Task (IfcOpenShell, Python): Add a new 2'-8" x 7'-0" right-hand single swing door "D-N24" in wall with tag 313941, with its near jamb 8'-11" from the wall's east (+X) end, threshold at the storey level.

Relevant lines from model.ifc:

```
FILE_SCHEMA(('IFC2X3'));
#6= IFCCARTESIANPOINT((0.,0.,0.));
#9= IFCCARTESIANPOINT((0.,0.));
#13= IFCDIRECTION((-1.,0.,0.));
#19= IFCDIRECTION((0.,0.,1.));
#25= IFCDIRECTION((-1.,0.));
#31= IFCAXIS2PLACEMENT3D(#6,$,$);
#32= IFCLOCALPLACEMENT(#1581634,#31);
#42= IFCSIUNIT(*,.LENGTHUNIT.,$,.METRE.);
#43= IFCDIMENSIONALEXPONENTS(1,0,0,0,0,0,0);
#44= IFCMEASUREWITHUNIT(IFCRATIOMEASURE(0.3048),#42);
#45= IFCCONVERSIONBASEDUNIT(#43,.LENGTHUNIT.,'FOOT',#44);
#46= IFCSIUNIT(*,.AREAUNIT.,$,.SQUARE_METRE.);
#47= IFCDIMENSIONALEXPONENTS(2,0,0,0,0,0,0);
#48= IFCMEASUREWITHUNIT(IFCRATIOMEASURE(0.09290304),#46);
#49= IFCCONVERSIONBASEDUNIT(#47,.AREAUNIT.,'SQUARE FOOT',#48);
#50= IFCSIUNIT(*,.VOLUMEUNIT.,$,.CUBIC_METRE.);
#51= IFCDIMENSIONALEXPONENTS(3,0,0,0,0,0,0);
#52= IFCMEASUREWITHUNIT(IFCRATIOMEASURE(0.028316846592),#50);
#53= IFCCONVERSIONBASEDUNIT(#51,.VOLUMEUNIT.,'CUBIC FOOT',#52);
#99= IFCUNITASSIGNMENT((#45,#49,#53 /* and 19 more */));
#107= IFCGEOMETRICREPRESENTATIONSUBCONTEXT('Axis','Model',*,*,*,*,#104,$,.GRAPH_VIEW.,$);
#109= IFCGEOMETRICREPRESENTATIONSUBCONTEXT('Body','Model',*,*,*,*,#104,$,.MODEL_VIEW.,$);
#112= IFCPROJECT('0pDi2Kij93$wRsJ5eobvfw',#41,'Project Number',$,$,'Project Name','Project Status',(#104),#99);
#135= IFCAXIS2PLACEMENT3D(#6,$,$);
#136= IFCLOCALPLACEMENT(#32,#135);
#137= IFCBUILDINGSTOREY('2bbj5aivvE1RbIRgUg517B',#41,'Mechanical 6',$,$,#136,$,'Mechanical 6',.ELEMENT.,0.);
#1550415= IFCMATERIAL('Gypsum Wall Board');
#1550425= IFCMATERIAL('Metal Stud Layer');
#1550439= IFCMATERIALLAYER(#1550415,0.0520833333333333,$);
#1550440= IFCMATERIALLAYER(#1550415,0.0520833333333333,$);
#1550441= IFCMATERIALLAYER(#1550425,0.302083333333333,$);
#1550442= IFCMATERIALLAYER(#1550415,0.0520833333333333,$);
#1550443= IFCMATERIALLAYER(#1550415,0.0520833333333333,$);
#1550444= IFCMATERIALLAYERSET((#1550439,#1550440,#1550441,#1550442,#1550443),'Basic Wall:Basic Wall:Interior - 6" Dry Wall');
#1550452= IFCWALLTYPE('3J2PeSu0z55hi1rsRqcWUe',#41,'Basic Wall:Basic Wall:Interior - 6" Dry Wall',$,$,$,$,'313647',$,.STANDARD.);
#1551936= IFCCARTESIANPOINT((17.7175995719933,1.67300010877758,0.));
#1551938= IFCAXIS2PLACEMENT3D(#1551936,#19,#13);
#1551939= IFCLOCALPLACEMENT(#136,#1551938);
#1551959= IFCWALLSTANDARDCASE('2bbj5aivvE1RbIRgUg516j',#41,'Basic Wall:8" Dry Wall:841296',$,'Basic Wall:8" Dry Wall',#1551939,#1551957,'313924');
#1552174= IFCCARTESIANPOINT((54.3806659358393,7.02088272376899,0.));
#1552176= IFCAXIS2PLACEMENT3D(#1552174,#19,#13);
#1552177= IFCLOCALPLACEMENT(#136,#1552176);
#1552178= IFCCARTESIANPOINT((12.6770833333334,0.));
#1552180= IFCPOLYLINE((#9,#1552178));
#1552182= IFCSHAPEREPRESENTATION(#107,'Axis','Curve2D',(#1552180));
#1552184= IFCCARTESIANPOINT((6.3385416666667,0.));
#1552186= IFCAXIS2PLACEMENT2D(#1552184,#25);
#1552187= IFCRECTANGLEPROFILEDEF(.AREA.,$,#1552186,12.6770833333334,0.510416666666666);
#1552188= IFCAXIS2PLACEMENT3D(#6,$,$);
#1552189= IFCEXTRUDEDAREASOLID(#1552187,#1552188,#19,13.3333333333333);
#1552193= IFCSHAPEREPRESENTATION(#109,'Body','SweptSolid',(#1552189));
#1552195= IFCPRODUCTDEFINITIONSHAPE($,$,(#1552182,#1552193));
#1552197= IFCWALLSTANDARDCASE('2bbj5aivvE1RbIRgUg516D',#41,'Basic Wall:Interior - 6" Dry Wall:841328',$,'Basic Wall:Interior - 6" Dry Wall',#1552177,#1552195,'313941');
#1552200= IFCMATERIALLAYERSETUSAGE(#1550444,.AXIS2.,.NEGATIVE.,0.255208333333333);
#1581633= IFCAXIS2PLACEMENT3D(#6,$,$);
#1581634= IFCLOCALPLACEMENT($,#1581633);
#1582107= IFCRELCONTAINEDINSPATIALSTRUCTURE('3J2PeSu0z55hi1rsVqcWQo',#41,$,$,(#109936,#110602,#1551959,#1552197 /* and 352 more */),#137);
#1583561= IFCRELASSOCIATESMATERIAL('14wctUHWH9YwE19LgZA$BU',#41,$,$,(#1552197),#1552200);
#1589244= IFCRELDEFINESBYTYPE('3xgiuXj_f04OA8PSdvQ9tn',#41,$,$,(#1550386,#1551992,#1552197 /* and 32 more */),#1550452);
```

```python
import numpy as np
import ifcopenshell
import ifcopenshell.api.feature
import ifcopenshell.api.geometry
import ifcopenshell.api.root
import ifcopenshell.api.spatial
import ifcopenshell.api.type
import ifcopenshell.geom
import ifcopenshell.util.element
import ifcopenshell.util.placement
import ifcopenshell.util.representation
import ifcopenshell.util.shape
import ifcopenshell.util.unit

model = ifcopenshell.open("model.ifc")
unit_scale = ifcopenshell.util.unit.calculate_unit_scale(model)
settings = ifcopenshell.geom.settings()


def volume(element):
    """Net volume in cubic metres, openings subtracted."""
    shape = ifcopenshell.geom.create_shape(settings, element)
    return ifcopenshell.util.shape.get_volume(shape.geometry)


wall = model.by_guid("2bbj5aivvE1RbIRgUg516D")
storey = ifcopenshell.util.element.get_container(wall, ifc_class="IfcBuildingStorey")
context = ifcopenshell.util.representation.get_context(model, "Model", "Body", "MODEL_VIEW")
before = volume(wall)

width, height, from_end, sill = 0.8128, 2.1336, 2.7178, 0.0  # metres

# The wall runs along its own X axis, and the end named is its -X end.
wall_shape = ifcopenshell.geom.create_shape(settings, wall)
x, y, z = ifcopenshell.util.shape.get_vertices(wall_shape.geometry).T
start = x.min() + from_end
face, thickness = float(y.min()), float(y.max() - y.min())
wall_matrix = ifcopenshell.util.placement.get_local_placement(wall.ObjectPlacement)
level = ifcopenshell.util.placement.get_local_placement(storey.ObjectPlacement)[2, 3]


def in_wall(x, y):
    """Placement at x, y metres in the wall's axes, at sill height."""
    matrix = wall_matrix.copy()
    matrix[:, 3] = wall_matrix @ np.array([x / unit_scale, y / unit_scale, 0.0, 1.0])
    matrix[2, 3] = level + sill / unit_scale
    return matrix


# Opening: a box that overshoots both wall faces by 50 mm.
opening = ifcopenshell.api.root.create_entity(model, ifc_class="IfcOpeningElement")
box = ifcopenshell.api.geometry.add_wall_representation(
    model, context=context, length=width, height=height, thickness=thickness + 0.1
)
ifcopenshell.api.geometry.assign_representation(model, product=opening, representation=box)
ifcopenshell.api.geometry.edit_object_placement(model, product=opening, matrix=in_wall(start, face - 0.05), is_si=False)
ifcopenshell.api.feature.add_feature(model, feature=opening, element=wall)

door = ifcopenshell.api.root.create_entity(model, ifc_class="IfcDoor", name="D-N24")
door.OverallWidth, door.OverallHeight = width / unit_scale, height / unit_scale
body = ifcopenshell.api.geometry.add_door_representation(
    model,
    context=context,
    overall_width=door.OverallWidth,
    overall_height=door.OverallHeight,
    operation_type="SINGLE_SWING_RIGHT",
    lining_properties={"LiningDepth": thickness / unit_scale, "ThresholdDepth": thickness / unit_scale},
)
ifcopenshell.api.geometry.assign_representation(model, product=door, representation=body)
ifcopenshell.api.spatial.assign_container(model, products=[door], relating_structure=storey)
fills = ifcopenshell.api.feature.add_filling(model, opening=opening, element=door)
fills.OwnerHistory = door.OwnerHistory  # required in IFC2X3

# IFC2X3 keeps the operation on the door style.
style = ifcopenshell.api.root.create_entity(model, ifc_class="IfcDoorStyle", name="D-N24")
style.OperationType, style.ConstructionType = "SINGLE_SWING_RIGHT", "NOTDEFINED"
style.ParameterTakesPrecedence = style.Sizeable = False
ifcopenshell.api.type.assign_type(model, related_objects=[door], relating_type=style)

# The lining spans the wall, so the door starts at the wall face.
ifcopenshell.api.geometry.edit_object_placement(model, product=door, matrix=in_wall(start, face), is_si=False)

after = volume(wall)

print(f"wall volume {before:.3f} -> {after:.3f} m3")

model.write("model_rev.ifc")
```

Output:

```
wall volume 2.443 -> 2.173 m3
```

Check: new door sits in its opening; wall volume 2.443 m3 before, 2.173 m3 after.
